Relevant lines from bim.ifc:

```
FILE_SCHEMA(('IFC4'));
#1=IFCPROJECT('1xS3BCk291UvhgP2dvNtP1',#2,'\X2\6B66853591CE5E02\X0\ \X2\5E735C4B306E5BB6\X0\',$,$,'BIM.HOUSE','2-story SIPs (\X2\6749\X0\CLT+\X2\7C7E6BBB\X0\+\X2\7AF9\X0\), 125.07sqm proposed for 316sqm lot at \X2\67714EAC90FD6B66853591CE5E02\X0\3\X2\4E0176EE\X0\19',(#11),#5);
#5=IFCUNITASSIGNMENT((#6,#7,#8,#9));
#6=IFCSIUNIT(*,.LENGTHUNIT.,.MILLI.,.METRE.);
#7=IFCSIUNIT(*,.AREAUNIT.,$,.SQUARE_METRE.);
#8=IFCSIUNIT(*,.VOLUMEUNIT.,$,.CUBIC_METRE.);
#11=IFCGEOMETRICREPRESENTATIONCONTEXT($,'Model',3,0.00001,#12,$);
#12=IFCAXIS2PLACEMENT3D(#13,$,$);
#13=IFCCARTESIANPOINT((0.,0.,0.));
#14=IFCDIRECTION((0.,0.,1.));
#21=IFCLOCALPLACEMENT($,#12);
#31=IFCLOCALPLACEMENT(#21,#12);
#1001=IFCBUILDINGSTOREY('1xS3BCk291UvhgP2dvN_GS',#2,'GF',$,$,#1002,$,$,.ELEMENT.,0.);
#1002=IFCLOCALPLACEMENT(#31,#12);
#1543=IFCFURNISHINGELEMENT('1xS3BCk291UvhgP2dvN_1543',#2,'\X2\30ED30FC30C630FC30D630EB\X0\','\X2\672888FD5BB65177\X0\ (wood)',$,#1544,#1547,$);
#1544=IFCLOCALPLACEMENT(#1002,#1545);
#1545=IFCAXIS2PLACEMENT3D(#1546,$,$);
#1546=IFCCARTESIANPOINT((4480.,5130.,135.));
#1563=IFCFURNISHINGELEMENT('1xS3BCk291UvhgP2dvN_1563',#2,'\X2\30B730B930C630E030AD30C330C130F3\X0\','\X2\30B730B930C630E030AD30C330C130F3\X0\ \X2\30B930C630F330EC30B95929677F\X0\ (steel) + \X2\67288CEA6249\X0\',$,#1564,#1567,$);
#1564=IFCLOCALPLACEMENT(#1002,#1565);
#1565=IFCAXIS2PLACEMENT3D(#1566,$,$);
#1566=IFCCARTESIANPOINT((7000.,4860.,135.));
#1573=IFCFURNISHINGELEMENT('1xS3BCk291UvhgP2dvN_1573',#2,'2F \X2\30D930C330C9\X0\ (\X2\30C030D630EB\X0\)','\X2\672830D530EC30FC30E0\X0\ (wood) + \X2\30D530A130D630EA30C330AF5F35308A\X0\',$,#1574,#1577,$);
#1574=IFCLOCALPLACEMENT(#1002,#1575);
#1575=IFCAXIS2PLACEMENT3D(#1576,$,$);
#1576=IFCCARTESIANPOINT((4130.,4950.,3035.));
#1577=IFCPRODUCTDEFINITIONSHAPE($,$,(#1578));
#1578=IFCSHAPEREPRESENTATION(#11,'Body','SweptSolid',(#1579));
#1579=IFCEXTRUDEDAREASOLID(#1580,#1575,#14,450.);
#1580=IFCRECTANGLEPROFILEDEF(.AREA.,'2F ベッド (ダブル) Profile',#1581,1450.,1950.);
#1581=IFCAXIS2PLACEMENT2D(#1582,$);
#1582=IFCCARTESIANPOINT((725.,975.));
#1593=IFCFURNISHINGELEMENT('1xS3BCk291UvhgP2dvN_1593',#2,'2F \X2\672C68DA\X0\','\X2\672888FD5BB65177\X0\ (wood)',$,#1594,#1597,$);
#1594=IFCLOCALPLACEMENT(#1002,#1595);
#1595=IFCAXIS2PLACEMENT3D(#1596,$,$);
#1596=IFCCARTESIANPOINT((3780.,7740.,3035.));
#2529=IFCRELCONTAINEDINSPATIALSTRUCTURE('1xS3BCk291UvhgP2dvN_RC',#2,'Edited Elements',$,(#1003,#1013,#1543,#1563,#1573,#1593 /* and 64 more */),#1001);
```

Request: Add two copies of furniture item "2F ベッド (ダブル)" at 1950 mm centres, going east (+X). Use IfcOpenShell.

```python
import numpy as np
import ifcopenshell
import ifcopenshell.api.geometry
import ifcopenshell.api.root
import ifcopenshell.util.element
import ifcopenshell.util.placement

model = ifcopenshell.open("bim.ifc")


def reuse_history(source, copy):
    """copy_class also copies each property set's owner history, people and application; keep the originals."""
    for rel in copy.IsDefinedBy:
        if rel.is_a("IfcRelDefinesByProperties") and (history := rel.RelatingPropertyDefinition.OwnerHistory):
            rel.RelatingPropertyDefinition.OwnerHistory = source.OwnerHistory
            ifcopenshell.util.element.remove_deep2(model, history)


source = model.by_guid("1xS3BCk291UvhgP2dvN_1573")
base = ifcopenshell.util.placement.get_local_placement(source.ObjectPlacement)
step = np.array([1.0, 0.0, 0.0]) * 1950.0

for i in range(1, 3):
    copy = ifcopenshell.api.root.copy_class(model, product=source)
    copy.Representation = ifcopenshell.util.element.copy_deep(
        model, source.Representation, exclude=["IfcGeometricRepresentationContext", "IfcRepresentationMap"]
    )
    reuse_history(source, copy)
    matrix = base.copy()
    matrix[:3, 3] += i * step
    print("added at", matrix[:3, 3].round(3) + 0.0)
    ifcopenshell.api.geometry.edit_object_placement(model, product=copy, matrix=matrix, is_si=False)

model.write("bim_updated.ifc")
```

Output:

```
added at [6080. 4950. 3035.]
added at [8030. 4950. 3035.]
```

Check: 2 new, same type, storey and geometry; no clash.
